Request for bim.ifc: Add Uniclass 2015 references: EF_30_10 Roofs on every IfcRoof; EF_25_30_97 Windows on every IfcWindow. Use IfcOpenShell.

First a look at what the model holds.

```python
import ifcopenshell

model = ifcopenshell.open("bim.ifc")
print(model.schema)
print("classifications:", [c.Name for c in model.by_type("IfcClassification")])
for ifc_class in ("IfcDoor", "IfcRoof", "IfcStair", "IfcWall", "IfcWindow"):
    print(ifc_class, len(model.by_type(ifc_class)))
```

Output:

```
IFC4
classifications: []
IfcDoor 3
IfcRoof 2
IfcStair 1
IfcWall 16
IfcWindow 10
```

```python
import ifcopenshell
import ifcopenshell.api.classification

model = ifcopenshell.open("bim.ifc")

system = ifcopenshell.api.classification.add_classification(model, classification="Uniclass 2015")

codes = {
    "IfcRoof": ("EF_30_10", "Roofs"),
    "IfcWindow": ("EF_25_30_97", "Windows"),
}
for ifc_class, (code, name) in codes.items():
    products = model.by_type(ifc_class)
    ifcopenshell.api.classification.add_reference(
        model, products=products, classification=system, identification=code, name=name
    )
    print(code, len(products))

model.write("bim_rev.ifc")
```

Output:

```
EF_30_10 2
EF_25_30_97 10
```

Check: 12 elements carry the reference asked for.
